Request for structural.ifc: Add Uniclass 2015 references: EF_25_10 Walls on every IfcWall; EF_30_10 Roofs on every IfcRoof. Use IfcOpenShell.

First a look at what the model holds.

```python
import ifcopenshell

model = ifcopenshell.open("structural.ifc")
print(model.schema)
print("classifications:", [c.Name for c in model.by_type("IfcClassification")])
for ifc_class in ("IfcDoor", "IfcRoof", "IfcStair", "IfcWall", "IfcWindow"):
    print(ifc_class, len(model.by_type(ifc_class)))
```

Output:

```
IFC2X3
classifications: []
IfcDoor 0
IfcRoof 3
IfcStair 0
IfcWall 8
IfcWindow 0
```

```python
import ifcopenshell
import ifcopenshell.api.classification

model = ifcopenshell.open("structural.ifc")

# IFC2X3 requires Source and Edition and has no link from the project to the system.
system = model.create_entity("IfcClassification", Source="NBS", Edition="2015", Name="Uniclass 2015")

codes = {
    "IfcWall": ("EF_25_10", "Walls"),
    "IfcRoof": ("EF_30_10", "Roofs"),
}
for ifc_class, (code, name) in codes.items():
    products = model.by_type(ifc_class)
    ifcopenshell.api.classification.add_reference(
        model, products=products, classification=system, identification=code, name=name
    )
    print(code, len(products))

model.write("structural_updated.ifc")
```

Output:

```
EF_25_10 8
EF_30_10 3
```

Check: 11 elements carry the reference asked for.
